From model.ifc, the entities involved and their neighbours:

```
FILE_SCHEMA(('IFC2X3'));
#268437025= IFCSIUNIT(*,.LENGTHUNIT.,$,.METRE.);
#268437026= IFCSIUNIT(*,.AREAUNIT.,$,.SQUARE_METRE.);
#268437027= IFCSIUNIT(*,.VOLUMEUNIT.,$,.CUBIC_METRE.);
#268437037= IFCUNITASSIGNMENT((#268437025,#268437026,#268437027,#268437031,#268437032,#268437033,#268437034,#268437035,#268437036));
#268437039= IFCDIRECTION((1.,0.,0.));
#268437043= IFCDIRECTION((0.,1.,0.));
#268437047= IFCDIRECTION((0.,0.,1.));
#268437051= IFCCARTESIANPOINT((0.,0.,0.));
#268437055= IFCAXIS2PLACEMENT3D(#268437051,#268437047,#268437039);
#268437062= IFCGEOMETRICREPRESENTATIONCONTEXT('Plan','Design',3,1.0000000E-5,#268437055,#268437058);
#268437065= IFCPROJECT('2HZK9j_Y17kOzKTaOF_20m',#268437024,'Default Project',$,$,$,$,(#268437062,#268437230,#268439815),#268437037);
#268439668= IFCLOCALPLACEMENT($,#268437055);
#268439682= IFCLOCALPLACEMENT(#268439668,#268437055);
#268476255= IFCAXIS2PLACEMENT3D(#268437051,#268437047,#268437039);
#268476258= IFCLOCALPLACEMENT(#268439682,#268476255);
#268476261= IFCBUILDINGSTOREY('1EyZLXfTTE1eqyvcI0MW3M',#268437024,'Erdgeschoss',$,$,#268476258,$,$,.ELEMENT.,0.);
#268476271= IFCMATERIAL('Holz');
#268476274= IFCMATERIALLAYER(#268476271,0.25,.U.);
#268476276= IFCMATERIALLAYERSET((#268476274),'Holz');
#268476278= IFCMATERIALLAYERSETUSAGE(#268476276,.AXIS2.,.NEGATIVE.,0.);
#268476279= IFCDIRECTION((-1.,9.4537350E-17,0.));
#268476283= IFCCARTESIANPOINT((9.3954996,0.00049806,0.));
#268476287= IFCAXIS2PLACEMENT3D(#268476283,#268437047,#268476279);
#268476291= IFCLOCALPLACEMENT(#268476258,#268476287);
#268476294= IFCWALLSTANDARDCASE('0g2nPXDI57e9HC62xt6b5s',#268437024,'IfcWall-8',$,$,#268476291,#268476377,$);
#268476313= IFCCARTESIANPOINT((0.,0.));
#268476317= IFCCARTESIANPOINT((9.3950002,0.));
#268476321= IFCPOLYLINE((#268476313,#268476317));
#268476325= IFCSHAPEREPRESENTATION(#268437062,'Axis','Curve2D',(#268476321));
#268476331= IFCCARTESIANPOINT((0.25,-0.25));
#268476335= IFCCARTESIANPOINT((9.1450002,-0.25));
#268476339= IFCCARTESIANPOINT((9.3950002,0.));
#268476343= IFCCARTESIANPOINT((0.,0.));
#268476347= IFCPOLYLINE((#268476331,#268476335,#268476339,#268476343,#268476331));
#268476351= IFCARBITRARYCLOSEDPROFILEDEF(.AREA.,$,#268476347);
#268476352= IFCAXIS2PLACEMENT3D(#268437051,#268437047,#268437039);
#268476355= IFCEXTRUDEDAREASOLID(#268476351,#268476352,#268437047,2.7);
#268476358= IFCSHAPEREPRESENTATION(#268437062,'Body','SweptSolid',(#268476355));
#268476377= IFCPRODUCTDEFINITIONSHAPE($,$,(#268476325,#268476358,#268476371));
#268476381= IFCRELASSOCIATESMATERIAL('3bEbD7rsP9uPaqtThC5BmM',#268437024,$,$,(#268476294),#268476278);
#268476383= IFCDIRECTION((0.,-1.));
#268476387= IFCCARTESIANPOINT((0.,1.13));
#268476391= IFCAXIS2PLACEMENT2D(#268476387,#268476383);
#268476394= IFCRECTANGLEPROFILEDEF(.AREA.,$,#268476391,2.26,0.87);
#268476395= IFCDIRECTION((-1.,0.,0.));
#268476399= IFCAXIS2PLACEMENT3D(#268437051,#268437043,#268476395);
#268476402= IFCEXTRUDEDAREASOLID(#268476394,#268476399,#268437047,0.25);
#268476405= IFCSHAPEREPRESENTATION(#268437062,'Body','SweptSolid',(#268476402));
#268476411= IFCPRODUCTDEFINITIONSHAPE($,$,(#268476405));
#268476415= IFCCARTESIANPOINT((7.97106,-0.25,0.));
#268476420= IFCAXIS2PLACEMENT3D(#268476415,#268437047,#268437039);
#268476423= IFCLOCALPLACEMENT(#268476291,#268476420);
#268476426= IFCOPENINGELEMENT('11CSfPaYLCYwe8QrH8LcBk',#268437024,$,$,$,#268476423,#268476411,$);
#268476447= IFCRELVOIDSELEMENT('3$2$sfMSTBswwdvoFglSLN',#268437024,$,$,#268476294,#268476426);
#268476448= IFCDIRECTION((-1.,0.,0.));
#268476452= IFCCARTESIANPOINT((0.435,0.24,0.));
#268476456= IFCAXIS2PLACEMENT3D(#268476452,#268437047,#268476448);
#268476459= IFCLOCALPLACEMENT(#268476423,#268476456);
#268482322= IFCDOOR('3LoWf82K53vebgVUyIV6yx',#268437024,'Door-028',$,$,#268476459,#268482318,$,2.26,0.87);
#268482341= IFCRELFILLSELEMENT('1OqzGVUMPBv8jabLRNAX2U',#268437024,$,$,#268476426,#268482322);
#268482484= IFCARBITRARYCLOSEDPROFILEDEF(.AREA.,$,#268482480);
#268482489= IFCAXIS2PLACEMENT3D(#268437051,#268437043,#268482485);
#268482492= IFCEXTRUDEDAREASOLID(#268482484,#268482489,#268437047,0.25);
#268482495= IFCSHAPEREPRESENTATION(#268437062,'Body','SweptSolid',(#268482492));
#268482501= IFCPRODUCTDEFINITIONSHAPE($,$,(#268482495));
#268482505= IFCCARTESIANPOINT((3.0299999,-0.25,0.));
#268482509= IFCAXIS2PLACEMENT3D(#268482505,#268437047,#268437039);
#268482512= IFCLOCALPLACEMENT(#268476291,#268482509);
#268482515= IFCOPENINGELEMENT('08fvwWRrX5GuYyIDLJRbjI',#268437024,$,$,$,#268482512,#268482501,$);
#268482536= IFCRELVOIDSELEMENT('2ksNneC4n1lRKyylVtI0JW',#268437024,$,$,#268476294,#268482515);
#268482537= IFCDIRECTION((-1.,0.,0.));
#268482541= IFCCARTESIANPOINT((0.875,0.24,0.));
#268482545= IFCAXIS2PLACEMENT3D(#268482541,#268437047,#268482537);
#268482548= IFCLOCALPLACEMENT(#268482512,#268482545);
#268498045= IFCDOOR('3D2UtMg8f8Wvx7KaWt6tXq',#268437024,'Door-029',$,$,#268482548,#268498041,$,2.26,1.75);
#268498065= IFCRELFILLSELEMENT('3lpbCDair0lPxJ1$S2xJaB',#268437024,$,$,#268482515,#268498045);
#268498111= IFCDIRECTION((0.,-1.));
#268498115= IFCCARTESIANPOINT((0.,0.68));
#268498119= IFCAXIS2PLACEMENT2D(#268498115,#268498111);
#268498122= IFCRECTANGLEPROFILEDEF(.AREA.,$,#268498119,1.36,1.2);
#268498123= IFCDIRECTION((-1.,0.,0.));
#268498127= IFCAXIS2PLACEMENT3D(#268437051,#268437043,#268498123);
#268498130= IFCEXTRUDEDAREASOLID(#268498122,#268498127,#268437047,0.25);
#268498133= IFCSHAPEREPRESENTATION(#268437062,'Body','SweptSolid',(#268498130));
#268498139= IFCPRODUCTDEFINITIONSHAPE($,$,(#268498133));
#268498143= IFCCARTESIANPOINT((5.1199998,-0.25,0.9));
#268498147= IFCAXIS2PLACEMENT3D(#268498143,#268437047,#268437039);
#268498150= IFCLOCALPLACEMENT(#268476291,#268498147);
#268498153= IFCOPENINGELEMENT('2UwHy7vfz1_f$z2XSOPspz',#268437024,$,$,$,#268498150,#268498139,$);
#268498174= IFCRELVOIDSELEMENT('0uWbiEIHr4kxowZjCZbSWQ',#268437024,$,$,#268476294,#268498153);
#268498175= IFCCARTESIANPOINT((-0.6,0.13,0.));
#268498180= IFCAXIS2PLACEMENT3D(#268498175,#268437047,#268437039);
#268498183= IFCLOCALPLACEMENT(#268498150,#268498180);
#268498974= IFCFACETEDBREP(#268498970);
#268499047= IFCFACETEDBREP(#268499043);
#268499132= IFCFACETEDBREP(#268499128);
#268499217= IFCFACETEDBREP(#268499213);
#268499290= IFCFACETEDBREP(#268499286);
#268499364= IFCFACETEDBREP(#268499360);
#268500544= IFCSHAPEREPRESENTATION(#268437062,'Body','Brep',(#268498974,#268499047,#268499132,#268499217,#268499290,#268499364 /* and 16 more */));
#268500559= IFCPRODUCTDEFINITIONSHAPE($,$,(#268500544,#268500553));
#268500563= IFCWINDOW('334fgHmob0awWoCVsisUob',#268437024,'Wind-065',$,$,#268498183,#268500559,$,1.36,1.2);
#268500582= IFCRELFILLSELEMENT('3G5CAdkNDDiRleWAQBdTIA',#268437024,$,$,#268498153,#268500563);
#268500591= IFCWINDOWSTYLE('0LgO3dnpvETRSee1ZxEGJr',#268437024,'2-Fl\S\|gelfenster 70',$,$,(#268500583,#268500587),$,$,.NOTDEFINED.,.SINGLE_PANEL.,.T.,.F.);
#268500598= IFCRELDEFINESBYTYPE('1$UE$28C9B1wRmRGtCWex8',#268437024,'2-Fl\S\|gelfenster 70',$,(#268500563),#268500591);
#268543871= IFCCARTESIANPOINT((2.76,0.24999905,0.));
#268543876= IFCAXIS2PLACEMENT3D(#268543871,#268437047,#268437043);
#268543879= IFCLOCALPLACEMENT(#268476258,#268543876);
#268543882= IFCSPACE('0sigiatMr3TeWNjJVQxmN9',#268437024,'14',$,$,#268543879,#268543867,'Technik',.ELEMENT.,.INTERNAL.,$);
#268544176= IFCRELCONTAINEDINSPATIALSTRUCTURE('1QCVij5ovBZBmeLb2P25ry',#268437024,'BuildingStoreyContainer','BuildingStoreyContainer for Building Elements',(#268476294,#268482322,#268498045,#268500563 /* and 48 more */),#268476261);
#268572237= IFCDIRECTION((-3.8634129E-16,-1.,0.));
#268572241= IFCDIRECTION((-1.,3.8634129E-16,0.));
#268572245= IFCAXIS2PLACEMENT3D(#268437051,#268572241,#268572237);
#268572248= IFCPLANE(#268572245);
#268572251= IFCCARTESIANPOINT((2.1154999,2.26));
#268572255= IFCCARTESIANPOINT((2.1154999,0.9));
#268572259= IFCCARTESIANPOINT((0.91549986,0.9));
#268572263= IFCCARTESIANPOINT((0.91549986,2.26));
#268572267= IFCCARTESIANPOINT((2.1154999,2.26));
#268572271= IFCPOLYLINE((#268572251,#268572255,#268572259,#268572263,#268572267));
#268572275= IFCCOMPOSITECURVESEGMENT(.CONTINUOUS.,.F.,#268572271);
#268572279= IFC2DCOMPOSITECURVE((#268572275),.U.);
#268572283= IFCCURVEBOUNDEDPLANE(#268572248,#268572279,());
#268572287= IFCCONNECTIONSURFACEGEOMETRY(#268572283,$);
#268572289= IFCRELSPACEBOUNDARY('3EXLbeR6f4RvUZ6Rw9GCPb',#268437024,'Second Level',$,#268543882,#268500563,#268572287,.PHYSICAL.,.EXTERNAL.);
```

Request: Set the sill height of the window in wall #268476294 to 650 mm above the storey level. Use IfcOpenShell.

```python
import numpy as np
import ifcopenshell
import ifcopenshell.api.geometry
import ifcopenshell.geom
import ifcopenshell.util.element
import ifcopenshell.util.placement
import ifcopenshell.util.shape
import ifcopenshell.util.unit

model = ifcopenshell.open("model.ifc")
unit_scale = ifcopenshell.util.unit.calculate_unit_scale(model)

window = model.by_guid("334fgHmob0awWoCVsisUob")
opening = window.FillsVoids[0].RelatingOpeningElement
storey = ifcopenshell.util.element.get_container(window, ifc_class="IfcBuildingStorey")
level = ifcopenshell.util.placement.get_local_placement(storey.ObjectPlacement)[2, 3]

# The opening's origin need not be at the sill, so measure its lowest point.
shape = ifcopenshell.geom.create_shape(ifcopenshell.geom.settings(), opening)
bottom = ifcopenshell.util.shape.get_shape_bottom_elevation(shape, shape.geometry) / unit_scale
dz = level + 0.65 / unit_scale - bottom

shift = np.array([0.0, 0.0, dz])
# The window is placed relative to its opening, so it follows when the opening moves.
matrix = ifcopenshell.util.placement.get_local_placement(opening.ObjectPlacement)
matrix[:3, 3] += shift
ifcopenshell.api.geometry.edit_object_placement(
    model, product=opening, matrix=matrix, is_si=False, should_transform_children=True
)

# Space boundary surfaces are stored in each space's coordinates; move them too.
for rel in window.ProvidesBoundaries:
    if not rel.ConnectionGeometry:
        continue
    surface = rel.ConnectionGeometry.SurfaceOnRelatingElement.BasisSurface
    space_matrix = ifcopenshell.util.placement.get_local_placement(rel.RelatingSpace.ObjectPlacement)
    point = np.array(surface.Position.Location.Coordinates) + space_matrix[:3, :3].T @ shift
    surface.Position = model.createIfcAxis2Placement3D(
        model.createIfcCartesianPoint(point.tolist()), surface.Position.Axis, surface.Position.RefDirection
    )

print(f"moved by {dz * unit_scale:+.3f} m")

model.write("model_v2.ifc")
```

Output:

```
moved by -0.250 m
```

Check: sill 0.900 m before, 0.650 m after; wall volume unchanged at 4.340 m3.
